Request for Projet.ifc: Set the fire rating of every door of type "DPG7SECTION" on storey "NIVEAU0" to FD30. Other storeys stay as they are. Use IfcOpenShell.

First a look at what the model holds.

```python
import ifcopenshell
import ifcopenshell.util.element

model = ifcopenshell.open("Projet.ifc")
print(model.schema)
storey = next(s for s in model.by_type("IfcBuildingStorey") if s.Name == "NIVEAU0")
doors = [e for e in ifcopenshell.util.element.get_decomposition(storey) if e.is_a("IfcDoor")]
seen = {}
for e in doors:
    element_type = ifcopenshell.util.element.get_type(e)
    key = (element_type.Name if element_type != e and element_type else None, ifcopenshell.util.element.get_pset(e, "Pset_DoorCommon", "FireRating"))
    seen[key] = seen.get(key, 0) + 1
for (name, value), count in sorted(seen.items(), key=str):
    print(count, "x", name, "|", value)
```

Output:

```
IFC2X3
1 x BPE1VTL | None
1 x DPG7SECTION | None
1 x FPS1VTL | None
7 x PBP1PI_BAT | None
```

```python
import ifcopenshell
import ifcopenshell.api.pset
import ifcopenshell.util.element

model = ifcopenshell.open("Projet.ifc")

storey = next(s for s in model.by_type("IfcBuildingStorey") if s.Name == "NIVEAU0")
doors = [e for e in ifcopenshell.util.element.get_decomposition(storey) if e.is_a("IfcDoor")]

count = 0
for e in doors:
    element_type = ifcopenshell.util.element.get_type(e)
    if element_type in (None, e) or element_type.Name != "DPG7SECTION":
        continue
    # add_pset returns the element's existing set when there is one.
    pset = ifcopenshell.api.pset.add_pset(model, product=e, name="Pset_DoorCommon")
    ifcopenshell.api.pset.edit_pset(model, pset=pset, properties={"FireRating": "FD30"})
    count += 1

print(count, "doors updated")

model.write("Projet_edited.ifc")
```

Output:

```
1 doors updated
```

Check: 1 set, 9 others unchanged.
